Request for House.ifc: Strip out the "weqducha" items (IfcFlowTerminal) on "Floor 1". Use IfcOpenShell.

First a look at what the model holds.

```python
import ifcopenshell
import ifcopenshell.util.element

model = ifcopenshell.open("House.ifc")
print(model.schema)
storey = next(s for s in model.by_type("IfcBuildingStorey") if s.Name == "Floor 1")
terminals = [e for e in ifcopenshell.util.element.get_decomposition(storey) if e.is_a("IfcFlowTerminal")]
seen = {}
for e in terminals:
    element_type = ifcopenshell.util.element.get_type(e)
    name = element_type.Name if element_type not in (None, e) else None
    seen[name] = seen.get(name, 0) + 1
for name, count in sorted(seen.items(), key=str):
    print(count, "x", name)
```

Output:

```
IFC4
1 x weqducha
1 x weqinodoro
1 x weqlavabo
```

```python
import ifcopenshell
import ifcopenshell.api.root
import ifcopenshell.util.element

model = ifcopenshell.open("House.ifc")

storey = next(s for s in model.by_type("IfcBuildingStorey") if s.Name == "Floor 1")
terminals = [e for e in ifcopenshell.util.element.get_decomposition(storey) if e.is_a("IfcFlowTerminal")]
targets = [e for e in terminals if (t := ifcopenshell.util.element.get_type(e)) not in (None, e) and t.Name == "weqducha"]

for e in targets:
    ifcopenshell.api.root.remove_product(model, product=e)
print(len(targets), "removed")

model.write("House_rev.ifc")
```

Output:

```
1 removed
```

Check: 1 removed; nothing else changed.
